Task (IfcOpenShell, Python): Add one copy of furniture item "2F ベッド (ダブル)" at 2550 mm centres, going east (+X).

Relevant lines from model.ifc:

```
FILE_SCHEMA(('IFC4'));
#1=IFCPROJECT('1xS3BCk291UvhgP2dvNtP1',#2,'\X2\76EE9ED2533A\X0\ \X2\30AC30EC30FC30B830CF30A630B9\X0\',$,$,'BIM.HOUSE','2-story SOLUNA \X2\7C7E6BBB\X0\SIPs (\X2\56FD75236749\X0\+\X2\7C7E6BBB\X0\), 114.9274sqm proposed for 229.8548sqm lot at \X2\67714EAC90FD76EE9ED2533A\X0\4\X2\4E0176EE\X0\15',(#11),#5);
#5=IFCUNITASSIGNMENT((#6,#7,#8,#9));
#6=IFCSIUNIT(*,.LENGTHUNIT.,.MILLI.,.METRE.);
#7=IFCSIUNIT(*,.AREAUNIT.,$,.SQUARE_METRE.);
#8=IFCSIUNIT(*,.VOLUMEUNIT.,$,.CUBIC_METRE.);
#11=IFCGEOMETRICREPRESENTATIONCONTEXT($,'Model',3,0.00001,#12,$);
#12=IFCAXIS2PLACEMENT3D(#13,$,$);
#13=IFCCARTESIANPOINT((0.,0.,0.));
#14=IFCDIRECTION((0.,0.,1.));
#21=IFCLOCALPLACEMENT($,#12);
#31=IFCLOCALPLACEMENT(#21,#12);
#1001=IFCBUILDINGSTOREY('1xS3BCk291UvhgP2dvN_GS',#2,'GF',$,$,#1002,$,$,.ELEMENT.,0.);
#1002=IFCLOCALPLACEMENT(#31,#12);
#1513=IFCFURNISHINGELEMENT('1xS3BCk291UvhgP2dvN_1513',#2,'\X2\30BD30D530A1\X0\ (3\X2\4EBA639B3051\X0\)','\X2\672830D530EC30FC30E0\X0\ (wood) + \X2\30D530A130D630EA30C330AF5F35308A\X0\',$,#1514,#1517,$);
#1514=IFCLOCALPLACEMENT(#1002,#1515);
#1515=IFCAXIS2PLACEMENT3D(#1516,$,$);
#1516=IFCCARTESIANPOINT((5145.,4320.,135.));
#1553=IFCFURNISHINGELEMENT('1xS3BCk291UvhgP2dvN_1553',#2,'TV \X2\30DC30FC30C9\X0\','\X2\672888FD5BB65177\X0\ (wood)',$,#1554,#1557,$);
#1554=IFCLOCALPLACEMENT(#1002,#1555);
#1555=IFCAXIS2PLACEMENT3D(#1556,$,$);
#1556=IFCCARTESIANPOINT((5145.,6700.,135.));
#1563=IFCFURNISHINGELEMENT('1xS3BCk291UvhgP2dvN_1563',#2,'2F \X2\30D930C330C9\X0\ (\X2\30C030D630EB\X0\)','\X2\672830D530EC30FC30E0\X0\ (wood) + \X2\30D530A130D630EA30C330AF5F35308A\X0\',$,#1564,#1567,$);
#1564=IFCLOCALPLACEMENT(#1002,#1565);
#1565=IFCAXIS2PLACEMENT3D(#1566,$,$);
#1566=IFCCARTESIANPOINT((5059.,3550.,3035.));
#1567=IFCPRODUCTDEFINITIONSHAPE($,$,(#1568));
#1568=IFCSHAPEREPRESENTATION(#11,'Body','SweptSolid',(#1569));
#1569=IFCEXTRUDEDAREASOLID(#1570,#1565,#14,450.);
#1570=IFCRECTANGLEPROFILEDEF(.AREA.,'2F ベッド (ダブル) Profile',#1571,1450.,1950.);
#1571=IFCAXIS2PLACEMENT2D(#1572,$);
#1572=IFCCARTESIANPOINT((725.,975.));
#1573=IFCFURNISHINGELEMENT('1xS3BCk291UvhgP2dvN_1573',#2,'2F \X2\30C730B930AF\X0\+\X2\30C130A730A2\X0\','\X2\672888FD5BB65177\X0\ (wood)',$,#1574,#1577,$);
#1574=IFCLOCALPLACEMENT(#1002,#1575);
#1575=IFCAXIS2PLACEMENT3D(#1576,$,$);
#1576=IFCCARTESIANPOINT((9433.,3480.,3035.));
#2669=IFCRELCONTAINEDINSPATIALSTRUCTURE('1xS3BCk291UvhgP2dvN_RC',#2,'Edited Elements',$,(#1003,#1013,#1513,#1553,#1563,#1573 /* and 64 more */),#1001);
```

```python
import numpy as np
import ifcopenshell
import ifcopenshell.api.geometry
import ifcopenshell.api.root
import ifcopenshell.util.element
import ifcopenshell.util.placement
import ifcopenshell.util.unit

model = ifcopenshell.open("model.ifc")
unit_scale = ifcopenshell.util.unit.calculate_unit_scale(model)


def reuse_history(source, copy):
    """copy_class also copies each property set's owner history, people and application; keep the originals."""
    for rel in copy.IsDefinedBy:
        if rel.is_a("IfcRelDefinesByProperties") and (history := rel.RelatingPropertyDefinition.OwnerHistory):
            rel.RelatingPropertyDefinition.OwnerHistory = source.OwnerHistory
            ifcopenshell.util.element.remove_deep2(model, history)


source = model.by_guid("1xS3BCk291UvhgP2dvN_1563")
base = ifcopenshell.util.placement.get_local_placement(source.ObjectPlacement)
step = np.array([1.0, 0.0, 0.0]) * 2.55 / unit_scale

for i in range(1, 2):
    copy = ifcopenshell.api.root.copy_class(model, product=source)
    copy.Representation = ifcopenshell.util.element.copy_deep(
        model, source.Representation, exclude=["IfcGeometricRepresentationContext", "IfcRepresentationMap"]
    )
    reuse_history(source, copy)
    matrix = base.copy()
    matrix[:3, 3] += i * step
    print("added at", matrix[:3, 3].round(3) + 0.0)
    ifcopenshell.api.geometry.edit_object_placement(model, product=copy, matrix=matrix, is_si=False)

model.write("model_rev.ifc")
```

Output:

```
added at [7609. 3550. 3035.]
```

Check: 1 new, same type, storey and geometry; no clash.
